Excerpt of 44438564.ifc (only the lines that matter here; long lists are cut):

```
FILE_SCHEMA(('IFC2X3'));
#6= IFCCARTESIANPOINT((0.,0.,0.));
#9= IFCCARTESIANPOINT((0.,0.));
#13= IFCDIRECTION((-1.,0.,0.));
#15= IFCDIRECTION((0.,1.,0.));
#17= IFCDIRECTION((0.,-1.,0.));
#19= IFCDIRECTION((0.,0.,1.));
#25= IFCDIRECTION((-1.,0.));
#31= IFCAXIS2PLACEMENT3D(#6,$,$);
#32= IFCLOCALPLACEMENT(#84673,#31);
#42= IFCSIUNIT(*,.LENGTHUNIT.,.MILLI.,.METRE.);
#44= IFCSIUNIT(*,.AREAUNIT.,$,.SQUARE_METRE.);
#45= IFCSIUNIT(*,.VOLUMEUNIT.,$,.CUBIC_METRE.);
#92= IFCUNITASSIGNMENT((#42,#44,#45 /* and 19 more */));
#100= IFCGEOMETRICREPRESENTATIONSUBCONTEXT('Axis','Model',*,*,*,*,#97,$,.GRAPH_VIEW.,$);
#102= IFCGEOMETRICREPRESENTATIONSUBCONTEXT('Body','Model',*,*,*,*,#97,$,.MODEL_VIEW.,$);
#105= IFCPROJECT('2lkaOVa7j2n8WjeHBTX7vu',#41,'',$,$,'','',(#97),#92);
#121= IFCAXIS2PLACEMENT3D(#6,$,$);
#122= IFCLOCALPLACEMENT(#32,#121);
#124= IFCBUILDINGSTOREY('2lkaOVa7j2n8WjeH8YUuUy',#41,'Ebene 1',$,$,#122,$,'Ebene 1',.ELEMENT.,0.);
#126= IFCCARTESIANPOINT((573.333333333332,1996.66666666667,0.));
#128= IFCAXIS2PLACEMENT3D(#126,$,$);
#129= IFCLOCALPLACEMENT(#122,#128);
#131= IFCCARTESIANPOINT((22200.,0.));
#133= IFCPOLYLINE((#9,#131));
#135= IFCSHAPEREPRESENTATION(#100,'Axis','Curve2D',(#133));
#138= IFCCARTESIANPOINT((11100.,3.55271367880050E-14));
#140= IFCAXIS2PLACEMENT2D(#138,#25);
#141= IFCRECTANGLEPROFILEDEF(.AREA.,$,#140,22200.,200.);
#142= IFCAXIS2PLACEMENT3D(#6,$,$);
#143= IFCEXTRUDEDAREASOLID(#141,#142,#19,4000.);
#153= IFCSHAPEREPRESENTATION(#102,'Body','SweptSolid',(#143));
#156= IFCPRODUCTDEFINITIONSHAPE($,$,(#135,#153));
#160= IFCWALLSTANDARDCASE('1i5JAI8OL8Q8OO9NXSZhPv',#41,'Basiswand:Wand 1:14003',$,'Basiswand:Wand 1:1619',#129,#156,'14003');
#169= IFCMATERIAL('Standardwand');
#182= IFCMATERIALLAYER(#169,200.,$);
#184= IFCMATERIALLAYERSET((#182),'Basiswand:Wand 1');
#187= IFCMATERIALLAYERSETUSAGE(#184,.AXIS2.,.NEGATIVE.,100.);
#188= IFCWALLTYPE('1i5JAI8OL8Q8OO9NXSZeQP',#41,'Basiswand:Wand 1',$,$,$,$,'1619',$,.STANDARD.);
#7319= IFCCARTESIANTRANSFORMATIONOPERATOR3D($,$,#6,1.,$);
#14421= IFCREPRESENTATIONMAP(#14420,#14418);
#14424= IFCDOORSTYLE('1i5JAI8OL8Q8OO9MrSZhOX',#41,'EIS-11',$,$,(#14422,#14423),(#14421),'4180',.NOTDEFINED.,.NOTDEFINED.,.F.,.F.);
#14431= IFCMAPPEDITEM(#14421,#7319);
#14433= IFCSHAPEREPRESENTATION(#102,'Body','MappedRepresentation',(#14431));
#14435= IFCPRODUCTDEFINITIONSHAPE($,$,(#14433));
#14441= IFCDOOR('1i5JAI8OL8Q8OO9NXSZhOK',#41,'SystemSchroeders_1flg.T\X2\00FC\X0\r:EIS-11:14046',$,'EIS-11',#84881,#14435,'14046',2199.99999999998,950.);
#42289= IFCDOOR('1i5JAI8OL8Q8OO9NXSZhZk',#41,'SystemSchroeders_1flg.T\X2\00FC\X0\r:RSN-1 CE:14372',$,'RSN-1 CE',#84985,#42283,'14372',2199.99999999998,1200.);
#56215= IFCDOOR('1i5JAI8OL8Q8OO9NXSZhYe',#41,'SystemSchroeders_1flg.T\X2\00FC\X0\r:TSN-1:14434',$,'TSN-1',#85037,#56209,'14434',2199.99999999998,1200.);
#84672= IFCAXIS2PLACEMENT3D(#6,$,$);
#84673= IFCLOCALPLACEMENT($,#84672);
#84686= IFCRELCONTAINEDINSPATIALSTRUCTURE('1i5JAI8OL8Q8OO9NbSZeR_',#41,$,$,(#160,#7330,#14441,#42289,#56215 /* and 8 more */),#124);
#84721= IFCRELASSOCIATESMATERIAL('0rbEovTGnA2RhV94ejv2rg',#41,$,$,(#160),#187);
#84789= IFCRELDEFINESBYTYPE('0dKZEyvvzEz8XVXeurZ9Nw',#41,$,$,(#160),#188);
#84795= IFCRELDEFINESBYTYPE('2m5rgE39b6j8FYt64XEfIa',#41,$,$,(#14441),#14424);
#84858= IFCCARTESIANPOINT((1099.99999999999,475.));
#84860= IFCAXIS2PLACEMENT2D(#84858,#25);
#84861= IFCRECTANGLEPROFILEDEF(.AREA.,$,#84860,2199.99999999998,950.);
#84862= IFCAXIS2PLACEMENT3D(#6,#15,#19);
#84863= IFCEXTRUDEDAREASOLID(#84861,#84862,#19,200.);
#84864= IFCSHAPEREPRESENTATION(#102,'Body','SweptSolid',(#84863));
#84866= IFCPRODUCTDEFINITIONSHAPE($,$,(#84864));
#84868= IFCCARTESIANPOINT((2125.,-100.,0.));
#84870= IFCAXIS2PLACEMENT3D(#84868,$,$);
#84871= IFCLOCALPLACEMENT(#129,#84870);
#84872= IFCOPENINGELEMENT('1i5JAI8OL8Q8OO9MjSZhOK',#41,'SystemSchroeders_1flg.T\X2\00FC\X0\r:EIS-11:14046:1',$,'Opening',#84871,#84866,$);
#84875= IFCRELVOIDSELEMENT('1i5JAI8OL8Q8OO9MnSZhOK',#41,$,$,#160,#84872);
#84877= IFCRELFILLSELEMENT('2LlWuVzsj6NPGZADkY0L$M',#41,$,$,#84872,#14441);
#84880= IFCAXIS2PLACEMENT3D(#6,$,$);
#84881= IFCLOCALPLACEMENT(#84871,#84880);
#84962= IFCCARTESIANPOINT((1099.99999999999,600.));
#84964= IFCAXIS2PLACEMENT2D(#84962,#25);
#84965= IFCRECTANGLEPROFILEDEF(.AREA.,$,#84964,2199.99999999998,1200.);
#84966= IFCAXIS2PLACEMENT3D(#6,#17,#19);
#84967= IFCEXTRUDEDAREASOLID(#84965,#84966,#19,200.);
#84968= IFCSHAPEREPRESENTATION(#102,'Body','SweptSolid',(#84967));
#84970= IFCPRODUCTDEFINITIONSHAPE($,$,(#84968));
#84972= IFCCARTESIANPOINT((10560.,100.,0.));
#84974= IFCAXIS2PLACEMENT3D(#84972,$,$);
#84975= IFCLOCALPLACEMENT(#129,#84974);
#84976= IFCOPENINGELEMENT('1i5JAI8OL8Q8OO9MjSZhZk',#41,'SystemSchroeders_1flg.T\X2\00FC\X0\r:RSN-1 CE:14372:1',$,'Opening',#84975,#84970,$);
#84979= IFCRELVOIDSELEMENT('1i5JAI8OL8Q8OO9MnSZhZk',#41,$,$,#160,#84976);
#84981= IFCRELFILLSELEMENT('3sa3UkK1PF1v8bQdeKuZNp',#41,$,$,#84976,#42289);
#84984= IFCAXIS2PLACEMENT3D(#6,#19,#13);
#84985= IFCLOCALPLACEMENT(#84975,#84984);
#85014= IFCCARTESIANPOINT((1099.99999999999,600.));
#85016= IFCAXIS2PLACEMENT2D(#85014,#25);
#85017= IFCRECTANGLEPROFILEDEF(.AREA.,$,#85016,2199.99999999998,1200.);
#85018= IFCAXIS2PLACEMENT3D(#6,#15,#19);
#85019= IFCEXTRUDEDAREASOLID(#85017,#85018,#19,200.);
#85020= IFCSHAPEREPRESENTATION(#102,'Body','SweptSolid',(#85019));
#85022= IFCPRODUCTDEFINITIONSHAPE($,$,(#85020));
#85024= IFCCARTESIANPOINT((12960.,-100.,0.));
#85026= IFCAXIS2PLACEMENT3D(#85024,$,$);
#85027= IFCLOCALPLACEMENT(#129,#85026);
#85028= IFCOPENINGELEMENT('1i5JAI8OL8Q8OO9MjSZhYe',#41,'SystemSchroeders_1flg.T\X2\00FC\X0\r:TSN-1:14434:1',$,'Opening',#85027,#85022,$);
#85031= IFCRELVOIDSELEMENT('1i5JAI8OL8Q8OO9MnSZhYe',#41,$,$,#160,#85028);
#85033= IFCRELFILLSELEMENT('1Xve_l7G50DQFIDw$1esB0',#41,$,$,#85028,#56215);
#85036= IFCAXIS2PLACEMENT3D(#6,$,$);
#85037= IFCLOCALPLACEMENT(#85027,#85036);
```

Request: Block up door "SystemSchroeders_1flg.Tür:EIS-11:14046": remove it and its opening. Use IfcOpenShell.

```python
import ifcopenshell
import ifcopenshell.api.feature
import ifcopenshell.api.root
import ifcopenshell.geom
import ifcopenshell.util.shape

model = ifcopenshell.open("44438564.ifc")
settings = ifcopenshell.geom.settings()


def volume(element):
    """Net volume in cubic metres, openings subtracted."""
    shape = ifcopenshell.geom.create_shape(settings, element)
    return ifcopenshell.util.shape.get_volume(shape.geometry)


door = model.by_guid("1i5JAI8OL8Q8OO9NXSZhOK")
opening = door.FillsVoids[0].RelatingOpeningElement
wall = opening.VoidsElements[0].RelatingBuildingElement
before = volume(wall)

ifcopenshell.api.root.remove_product(model, product=door)
ifcopenshell.api.feature.remove_feature(model, feature=opening)

after = volume(wall)

print(f"wall volume {before:.3f} -> {after:.3f} m3")

model.write("44438564_rev.ifc")
```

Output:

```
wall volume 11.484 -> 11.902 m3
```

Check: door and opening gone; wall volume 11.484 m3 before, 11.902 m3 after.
